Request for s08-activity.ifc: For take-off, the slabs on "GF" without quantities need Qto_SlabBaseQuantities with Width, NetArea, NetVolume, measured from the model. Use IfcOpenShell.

First a look at what the model holds.

```python
import ifcopenshell
import ifcopenshell.util.element
import ifcopenshell.util.unit

model = ifcopenshell.open("s08-activity.ifc")
print(model.schema)
for unit_type in ("LENGTHUNIT", "AREAUNIT", "VOLUMEUNIT"):
    print(unit_type, ifcopenshell.util.unit.calculate_unit_scale(model, unit_type))
storey = next(s for s in model.by_type("IfcBuildingStorey") if s.Name == "GF")
slabs = [e for e in ifcopenshell.util.element.get_decomposition(storey) if e.is_a("IfcSlab")]
for e in sorted(slabs, key=lambda e: e.id()):
    print(e.id(), e.is_a(), e.Name, list(ifcopenshell.util.element.get_psets(e, qtos_only=True)), sep=" | ")
```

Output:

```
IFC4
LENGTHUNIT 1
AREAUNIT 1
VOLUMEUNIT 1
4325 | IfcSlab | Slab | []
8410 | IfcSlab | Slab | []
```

```python
import ifcopenshell
import ifcopenshell.api.pset
import ifcopenshell.geom
import ifcopenshell.util.element
import ifcopenshell.util.shape
import ifcopenshell.util.unit

model = ifcopenshell.open("s08-activity.ifc")
unit_scale = ifcopenshell.util.unit.calculate_unit_scale(model)
area_scale = ifcopenshell.util.unit.calculate_unit_scale(model, "AREAUNIT")
volume_scale = ifcopenshell.util.unit.calculate_unit_scale(model, "VOLUMEUNIT")
settings = ifcopenshell.geom.settings()

storey = next(s for s in model.by_type("IfcBuildingStorey") if s.Name == "GF")
slabs = [e for e in ifcopenshell.util.element.get_decomposition(storey) if e.is_a("IfcSlab")]

for e in sorted(slabs, key=lambda e: e.id()):
    if ifcopenshell.util.element.get_psets(e, qtos_only=True, should_inherit=False):
        continue
    # Geometry comes back in metres, in the element's own axes.
    shape = ifcopenshell.geom.create_shape(settings, e)
    values = {
        "Width": ifcopenshell.util.shape.get_z(shape.geometry) / unit_scale,
        "NetArea": ifcopenshell.util.shape.get_footprint_area(shape.geometry) / area_scale,
        "NetVolume": ifcopenshell.util.shape.get_volume(shape.geometry) / volume_scale,
    }
    qto = ifcopenshell.api.pset.add_qto(model, product=e, name="Qto_SlabBaseQuantities")
    ifcopenshell.api.pset.edit_qto(model, qto=qto, properties=values)
    print(e.id(), {k: round(v, 3) for k, v in values.items()})

model.write("s08-activity-out.ifc")
```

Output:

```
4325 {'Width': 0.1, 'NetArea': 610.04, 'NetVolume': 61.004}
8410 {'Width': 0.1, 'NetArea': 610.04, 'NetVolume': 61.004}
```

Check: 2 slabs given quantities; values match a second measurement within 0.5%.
